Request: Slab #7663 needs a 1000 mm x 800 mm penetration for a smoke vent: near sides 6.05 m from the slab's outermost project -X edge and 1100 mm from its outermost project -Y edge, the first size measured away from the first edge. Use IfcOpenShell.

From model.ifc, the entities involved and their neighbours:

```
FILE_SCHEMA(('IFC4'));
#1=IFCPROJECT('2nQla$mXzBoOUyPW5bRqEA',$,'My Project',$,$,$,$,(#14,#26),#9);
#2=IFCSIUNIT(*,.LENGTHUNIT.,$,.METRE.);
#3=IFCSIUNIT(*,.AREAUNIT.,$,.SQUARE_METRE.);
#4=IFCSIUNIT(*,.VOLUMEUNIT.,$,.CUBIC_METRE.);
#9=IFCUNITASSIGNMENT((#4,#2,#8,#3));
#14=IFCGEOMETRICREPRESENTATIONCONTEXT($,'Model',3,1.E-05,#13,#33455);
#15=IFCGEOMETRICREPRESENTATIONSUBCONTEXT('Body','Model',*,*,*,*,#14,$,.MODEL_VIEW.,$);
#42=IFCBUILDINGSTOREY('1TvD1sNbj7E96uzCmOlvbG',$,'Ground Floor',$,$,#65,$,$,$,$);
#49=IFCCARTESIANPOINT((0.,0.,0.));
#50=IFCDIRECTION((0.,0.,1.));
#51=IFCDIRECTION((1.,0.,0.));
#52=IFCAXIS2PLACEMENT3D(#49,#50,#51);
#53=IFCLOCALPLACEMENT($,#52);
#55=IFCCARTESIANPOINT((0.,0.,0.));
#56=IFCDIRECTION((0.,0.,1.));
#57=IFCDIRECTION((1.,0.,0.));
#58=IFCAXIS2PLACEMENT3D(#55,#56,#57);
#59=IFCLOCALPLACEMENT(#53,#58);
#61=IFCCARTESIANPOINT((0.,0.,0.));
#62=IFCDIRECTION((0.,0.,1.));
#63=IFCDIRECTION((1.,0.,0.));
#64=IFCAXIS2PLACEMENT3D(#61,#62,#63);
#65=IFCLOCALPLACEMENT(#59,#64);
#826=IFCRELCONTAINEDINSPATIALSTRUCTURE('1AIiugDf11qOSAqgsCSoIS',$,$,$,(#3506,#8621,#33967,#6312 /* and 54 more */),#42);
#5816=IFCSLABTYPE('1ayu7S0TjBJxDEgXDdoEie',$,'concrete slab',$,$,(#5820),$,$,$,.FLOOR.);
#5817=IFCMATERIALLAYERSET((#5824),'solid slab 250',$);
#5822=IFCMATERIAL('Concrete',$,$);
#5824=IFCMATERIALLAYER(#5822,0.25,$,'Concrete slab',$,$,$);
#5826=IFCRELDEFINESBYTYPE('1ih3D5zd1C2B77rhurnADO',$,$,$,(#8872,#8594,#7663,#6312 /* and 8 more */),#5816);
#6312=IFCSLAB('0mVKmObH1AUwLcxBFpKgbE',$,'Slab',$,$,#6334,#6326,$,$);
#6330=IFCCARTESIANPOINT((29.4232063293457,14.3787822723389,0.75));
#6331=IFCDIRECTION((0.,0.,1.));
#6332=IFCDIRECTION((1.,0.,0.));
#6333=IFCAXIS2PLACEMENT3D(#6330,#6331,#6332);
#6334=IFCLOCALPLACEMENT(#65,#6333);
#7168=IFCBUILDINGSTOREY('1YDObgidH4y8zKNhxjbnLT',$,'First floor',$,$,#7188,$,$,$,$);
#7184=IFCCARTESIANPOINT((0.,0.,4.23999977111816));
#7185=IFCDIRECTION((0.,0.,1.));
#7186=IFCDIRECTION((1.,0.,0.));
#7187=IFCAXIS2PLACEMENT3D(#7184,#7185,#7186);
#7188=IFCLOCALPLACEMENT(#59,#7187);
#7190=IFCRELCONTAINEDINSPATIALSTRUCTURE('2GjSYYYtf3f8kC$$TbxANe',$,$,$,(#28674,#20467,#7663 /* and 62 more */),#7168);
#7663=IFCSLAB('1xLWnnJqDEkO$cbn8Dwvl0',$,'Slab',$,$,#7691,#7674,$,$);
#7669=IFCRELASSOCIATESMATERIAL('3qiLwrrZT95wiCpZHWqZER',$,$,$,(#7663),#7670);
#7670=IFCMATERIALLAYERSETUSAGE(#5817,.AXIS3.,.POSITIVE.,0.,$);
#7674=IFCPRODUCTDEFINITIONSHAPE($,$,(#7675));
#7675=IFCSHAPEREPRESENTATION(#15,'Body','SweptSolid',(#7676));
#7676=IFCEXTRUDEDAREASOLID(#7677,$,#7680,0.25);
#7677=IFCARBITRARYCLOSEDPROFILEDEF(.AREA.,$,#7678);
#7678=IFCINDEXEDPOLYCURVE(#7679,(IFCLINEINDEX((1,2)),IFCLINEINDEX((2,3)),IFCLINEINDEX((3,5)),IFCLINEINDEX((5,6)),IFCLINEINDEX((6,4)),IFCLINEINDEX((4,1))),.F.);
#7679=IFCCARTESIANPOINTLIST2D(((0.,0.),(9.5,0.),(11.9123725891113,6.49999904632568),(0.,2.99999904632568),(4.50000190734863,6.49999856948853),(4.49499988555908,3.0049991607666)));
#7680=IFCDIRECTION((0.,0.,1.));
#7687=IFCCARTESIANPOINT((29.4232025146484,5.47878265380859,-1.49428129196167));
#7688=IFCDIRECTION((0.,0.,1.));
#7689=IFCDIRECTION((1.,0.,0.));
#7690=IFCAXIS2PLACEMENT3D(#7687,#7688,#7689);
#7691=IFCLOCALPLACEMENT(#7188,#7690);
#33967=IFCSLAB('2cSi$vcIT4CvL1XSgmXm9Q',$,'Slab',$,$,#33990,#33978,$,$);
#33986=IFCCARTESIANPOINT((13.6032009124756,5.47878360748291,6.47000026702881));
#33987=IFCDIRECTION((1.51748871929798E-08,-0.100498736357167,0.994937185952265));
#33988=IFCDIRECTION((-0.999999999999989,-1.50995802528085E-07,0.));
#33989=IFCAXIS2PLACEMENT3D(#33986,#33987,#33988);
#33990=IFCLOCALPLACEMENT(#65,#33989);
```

```python
import numpy as np
import ifcopenshell
import ifcopenshell.api.feature
import ifcopenshell.api.geometry
import ifcopenshell.api.root
import ifcopenshell.geom
import ifcopenshell.util.placement
import ifcopenshell.util.representation
import ifcopenshell.util.shape
import ifcopenshell.util.unit

model = ifcopenshell.open("model.ifc")
unit_scale = ifcopenshell.util.unit.calculate_unit_scale(model)
settings = ifcopenshell.geom.settings()


def volume(element):
    """Net volume in cubic metres, openings subtracted."""
    shape = ifcopenshell.geom.create_shape(settings, element)
    return ifcopenshell.util.shape.get_volume(shape.geometry)


slab = model.by_guid("1xLWnnJqDEkO$cbn8Dwvl0")
before = volume(slab)

# Extent in the slab's own axes, in metres. The edges named are its -X and -Y sides.
slab_shape = ifcopenshell.geom.create_shape(settings, slab)
vertices = ifcopenshell.util.shape.get_vertices(slab_shape.geometry)
x_min, y_min, bottom = vertices.min(axis=0)
top = vertices[:, 2].max()

opening = ifcopenshell.api.root.create_entity(model, ifc_class="IfcOpeningElement", name="Smoke vent opening", predefined_type="OPENING")
context = ifcopenshell.util.representation.get_context(model, "Model", "Body", "MODEL_VIEW")
width, depth = 1, 0.8
outline = [(0.0, 0.0), (width, 0.0), (width, depth), (0.0, depth), (0.0, 0.0)]
# Overshoot both faces by 50 mm so the cut is clean.
shape = ifcopenshell.api.geometry.add_slab_representation(
    model, context=context, depth=top - bottom + 0.1, polyline=outline
)
ifcopenshell.api.geometry.assign_representation(model, product=opening, representation=shape)

matrix = ifcopenshell.util.placement.get_local_placement(slab.ObjectPlacement)
matrix[:, 3] = matrix @ np.append(np.array([x_min + 6.05, y_min + 1.1, bottom - 0.05]) / unit_scale, 1.0)
ifcopenshell.api.geometry.edit_object_placement(model, product=opening, matrix=matrix, is_si=False)
ifcopenshell.api.feature.add_feature(model, feature=opening, element=slab)

after = volume(slab)

print(f"slab volume {before:.3f} -> {after:.3f} m3")

model.write("model_rev.ifc")
```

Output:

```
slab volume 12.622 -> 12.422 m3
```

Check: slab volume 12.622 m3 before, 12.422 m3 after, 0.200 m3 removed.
